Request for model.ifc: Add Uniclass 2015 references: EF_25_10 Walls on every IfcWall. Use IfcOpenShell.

First a look at what the model holds.

```python
import ifcopenshell

model = ifcopenshell.open("model.ifc")
print(model.schema)
print("classifications:", [c.Name for c in model.by_type("IfcClassification")])
for ifc_class in ("IfcDoor", "IfcRoof", "IfcStair", "IfcWall", "IfcWindow"):
    print(ifc_class, len(model.by_type(ifc_class)))
```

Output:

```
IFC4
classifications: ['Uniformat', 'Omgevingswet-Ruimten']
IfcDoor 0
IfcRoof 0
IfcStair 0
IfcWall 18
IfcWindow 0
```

```python
import ifcopenshell
import ifcopenshell.api.classification

model = ifcopenshell.open("model.ifc")

system = ifcopenshell.api.classification.add_classification(model, classification="Uniclass 2015")

codes = {
    "IfcWall": ("EF_25_10", "Walls"),
}
for ifc_class, (code, name) in codes.items():
    products = model.by_type(ifc_class)
    ifcopenshell.api.classification.add_reference(
        model, products=products, classification=system, identification=code, name=name
    )
    print(code, len(products))

model.write("model_rev.ifc")
```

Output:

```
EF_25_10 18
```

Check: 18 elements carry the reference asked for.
